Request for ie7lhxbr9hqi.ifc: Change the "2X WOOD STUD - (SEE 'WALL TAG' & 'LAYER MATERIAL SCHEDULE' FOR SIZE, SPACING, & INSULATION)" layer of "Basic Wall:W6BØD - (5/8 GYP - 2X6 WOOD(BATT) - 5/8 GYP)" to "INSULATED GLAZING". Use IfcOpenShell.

First a look at what the model holds.

```python
import ifcopenshell
import ifcopenshell.util.element

model = ifcopenshell.open("ie7lhxbr9hqi.ifc")
print(model.schema)
for layer_set in model.by_type("IfcMaterialLayerSet"):
    if layer_set.LayerSetName == "Basic Wall:W6BØD - (5/8 GYP - 2X6 WOOD(BATT) - 5/8 GYP)":
        for layer in layer_set.MaterialLayers:
            print(layer.id(), layer.Material and layer.Material.Name, layer.LayerThickness, sep=" | ")
        print(len(ifcopenshell.util.element.get_elements_by_material(model, layer_set)), "elements and types use it")
print(sorted(m.Name for m in model.by_type("IfcMaterial") if m.Name)[:60])
```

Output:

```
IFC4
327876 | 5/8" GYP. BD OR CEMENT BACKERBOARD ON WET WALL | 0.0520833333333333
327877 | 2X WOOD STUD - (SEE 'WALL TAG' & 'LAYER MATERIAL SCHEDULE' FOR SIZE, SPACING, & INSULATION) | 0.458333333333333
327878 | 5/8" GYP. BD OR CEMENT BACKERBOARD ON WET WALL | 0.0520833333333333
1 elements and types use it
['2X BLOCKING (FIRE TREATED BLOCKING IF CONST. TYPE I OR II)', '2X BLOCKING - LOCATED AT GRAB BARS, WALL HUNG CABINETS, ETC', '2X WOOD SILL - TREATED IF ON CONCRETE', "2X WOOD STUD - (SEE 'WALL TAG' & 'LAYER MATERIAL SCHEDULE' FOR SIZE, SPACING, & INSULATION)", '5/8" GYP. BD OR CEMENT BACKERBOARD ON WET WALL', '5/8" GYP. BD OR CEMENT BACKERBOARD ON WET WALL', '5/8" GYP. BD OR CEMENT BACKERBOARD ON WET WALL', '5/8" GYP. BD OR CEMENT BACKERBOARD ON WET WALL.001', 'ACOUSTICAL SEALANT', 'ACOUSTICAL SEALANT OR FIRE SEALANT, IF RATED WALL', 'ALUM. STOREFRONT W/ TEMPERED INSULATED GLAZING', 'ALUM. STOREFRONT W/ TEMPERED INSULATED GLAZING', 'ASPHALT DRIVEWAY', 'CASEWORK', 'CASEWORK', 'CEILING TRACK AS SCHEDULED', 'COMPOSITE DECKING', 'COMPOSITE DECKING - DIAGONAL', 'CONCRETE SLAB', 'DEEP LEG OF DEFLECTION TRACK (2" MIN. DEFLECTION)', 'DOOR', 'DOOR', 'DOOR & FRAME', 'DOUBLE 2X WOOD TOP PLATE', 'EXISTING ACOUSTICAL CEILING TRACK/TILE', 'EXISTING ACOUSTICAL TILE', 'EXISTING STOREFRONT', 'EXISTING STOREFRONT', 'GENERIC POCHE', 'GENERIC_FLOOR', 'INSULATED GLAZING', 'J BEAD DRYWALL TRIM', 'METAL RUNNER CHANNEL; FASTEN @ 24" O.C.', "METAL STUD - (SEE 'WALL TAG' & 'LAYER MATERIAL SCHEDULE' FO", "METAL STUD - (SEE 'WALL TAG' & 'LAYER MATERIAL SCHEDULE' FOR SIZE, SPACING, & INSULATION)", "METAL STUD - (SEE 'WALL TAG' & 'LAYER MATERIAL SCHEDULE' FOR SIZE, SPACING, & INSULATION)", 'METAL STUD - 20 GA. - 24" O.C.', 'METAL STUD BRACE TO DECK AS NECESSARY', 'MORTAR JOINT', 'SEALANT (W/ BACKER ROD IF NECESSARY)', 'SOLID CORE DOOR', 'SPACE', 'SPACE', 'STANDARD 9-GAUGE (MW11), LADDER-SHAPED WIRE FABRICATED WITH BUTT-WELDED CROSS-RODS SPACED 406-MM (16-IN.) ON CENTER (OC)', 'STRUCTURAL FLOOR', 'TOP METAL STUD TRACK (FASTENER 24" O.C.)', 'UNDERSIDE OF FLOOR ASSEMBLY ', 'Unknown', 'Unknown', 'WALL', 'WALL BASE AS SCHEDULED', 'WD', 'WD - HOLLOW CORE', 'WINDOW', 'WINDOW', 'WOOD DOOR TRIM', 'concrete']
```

```python
import ifcopenshell
import ifcopenshell.api.material

model = ifcopenshell.open("ie7lhxbr9hqi.ifc")

layer_set = next(s for s in model.by_type("IfcMaterialLayerSet") if s.LayerSetName == "Basic Wall:W6BØD - (5/8 GYP - 2X6 WOOD(BATT) - 5/8 GYP)")
layer = next(l for l in layer_set.MaterialLayers if l.Material and l.Material.Name == "2X WOOD STUD - (SEE 'WALL TAG' & 'LAYER MATERIAL SCHEDULE' FOR SIZE, SPACING, & INSULATION)")
material = next(m for m in model.by_type("IfcMaterial") if m.Name == "INSULATED GLAZING")

# Point this one layer at the other material; renaming the old one would change it everywhere.
ifcopenshell.api.material.edit_layer(model, layer=layer, attributes={}, material=material)

print([l.Material.Name if l.Material else None for l in layer_set.MaterialLayers])

model.write("ie7lhxbr9hqi_rev.ifc")
```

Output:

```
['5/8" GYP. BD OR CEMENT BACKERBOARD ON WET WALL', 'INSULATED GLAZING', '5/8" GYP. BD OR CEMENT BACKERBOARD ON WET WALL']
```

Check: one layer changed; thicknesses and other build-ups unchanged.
